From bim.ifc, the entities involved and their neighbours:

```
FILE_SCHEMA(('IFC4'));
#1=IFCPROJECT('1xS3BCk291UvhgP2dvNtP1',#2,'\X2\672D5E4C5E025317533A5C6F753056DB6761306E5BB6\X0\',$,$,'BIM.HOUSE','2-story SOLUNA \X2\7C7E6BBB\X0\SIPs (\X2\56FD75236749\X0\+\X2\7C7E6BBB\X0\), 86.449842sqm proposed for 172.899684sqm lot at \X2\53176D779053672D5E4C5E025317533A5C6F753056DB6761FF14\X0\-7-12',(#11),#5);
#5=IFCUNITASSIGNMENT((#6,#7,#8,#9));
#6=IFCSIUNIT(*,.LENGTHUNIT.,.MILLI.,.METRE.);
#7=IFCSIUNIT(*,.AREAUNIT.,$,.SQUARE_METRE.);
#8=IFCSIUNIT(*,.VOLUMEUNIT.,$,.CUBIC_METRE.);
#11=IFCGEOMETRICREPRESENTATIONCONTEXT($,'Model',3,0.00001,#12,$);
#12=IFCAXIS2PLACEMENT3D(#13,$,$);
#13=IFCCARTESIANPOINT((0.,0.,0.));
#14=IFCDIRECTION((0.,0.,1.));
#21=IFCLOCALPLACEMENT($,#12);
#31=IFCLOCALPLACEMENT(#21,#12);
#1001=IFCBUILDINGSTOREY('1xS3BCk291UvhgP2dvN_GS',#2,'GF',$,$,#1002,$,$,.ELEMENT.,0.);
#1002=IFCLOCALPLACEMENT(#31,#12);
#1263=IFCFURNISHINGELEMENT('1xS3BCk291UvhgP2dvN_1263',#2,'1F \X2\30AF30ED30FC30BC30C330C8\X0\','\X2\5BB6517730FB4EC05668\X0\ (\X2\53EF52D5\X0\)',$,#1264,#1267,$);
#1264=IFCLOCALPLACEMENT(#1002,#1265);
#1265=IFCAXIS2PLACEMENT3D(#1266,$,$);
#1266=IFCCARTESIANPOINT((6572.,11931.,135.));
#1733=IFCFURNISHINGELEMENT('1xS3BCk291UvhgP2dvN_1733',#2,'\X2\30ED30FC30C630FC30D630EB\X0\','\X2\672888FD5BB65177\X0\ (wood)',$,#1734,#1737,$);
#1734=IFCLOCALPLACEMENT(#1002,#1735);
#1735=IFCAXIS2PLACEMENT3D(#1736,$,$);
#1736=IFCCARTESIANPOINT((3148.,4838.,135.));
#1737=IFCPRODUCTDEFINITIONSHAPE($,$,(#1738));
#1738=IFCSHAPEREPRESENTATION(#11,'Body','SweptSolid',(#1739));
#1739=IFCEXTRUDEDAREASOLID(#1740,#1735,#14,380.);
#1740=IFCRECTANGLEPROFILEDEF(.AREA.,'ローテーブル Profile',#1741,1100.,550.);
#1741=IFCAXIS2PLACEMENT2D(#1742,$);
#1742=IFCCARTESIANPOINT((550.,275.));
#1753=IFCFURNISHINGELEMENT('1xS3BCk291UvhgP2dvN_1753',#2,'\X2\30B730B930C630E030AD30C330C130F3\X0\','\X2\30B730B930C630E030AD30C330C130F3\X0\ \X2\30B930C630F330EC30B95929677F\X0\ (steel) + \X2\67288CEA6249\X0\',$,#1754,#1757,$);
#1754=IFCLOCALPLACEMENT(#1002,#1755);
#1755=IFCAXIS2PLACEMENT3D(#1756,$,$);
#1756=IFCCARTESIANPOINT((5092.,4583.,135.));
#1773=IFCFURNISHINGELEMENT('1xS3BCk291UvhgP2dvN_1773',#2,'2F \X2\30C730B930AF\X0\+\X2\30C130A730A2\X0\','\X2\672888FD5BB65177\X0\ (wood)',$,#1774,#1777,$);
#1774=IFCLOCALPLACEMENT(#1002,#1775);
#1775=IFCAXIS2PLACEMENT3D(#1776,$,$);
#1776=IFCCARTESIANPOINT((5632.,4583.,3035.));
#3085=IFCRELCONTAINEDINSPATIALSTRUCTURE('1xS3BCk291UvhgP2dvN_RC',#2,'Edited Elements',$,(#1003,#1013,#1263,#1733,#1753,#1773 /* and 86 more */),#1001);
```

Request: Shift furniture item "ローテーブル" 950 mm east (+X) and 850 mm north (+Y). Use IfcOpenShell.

```python
import ifcopenshell
import ifcopenshell.api.geometry
import ifcopenshell.util.placement

model = ifcopenshell.open("bim.ifc")

item = model.by_id(1733)
matrix = ifcopenshell.util.placement.get_local_placement(item.ObjectPlacement)
matrix[0, 3] += 950.0
matrix[1, 3] += 850.0
ifcopenshell.api.geometry.edit_object_placement(model, product=item, matrix=matrix, is_si=False)

print(ifcopenshell.util.placement.get_local_placement(item.ObjectPlacement).round(3) + 0.0)

model.write("bim_edited.ifc")
```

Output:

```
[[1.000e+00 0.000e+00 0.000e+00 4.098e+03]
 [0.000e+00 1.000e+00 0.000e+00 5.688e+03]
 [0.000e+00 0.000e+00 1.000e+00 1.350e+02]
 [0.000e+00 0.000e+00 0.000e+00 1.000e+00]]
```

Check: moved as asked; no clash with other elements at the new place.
